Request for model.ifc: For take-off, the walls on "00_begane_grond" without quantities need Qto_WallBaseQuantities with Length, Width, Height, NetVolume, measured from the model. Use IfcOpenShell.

First a look at what the model holds.

```python
import ifcopenshell
import ifcopenshell.util.element
import ifcopenshell.util.unit

model = ifcopenshell.open("model.ifc")
print(model.schema)
for unit_type in ("LENGTHUNIT", "AREAUNIT", "VOLUMEUNIT"):
    print(unit_type, ifcopenshell.util.unit.calculate_unit_scale(model, unit_type))
storey = next(s for s in model.by_type("IfcBuildingStorey") if s.Name == "00_begane_grond")
walls = [e for e in ifcopenshell.util.element.get_decomposition(storey) if e.is_a("IfcWall")]
for e in sorted(walls, key=lambda e: e.id()):
    print(e.id(), e.is_a(), e.Name, list(ifcopenshell.util.element.get_psets(e, qtos_only=True)), sep=" | ")
```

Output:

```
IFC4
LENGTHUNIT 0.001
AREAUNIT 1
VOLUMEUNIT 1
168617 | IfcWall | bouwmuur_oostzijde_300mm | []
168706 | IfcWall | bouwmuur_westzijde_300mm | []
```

```python
import ifcopenshell
import ifcopenshell.api.pset
import ifcopenshell.geom
import ifcopenshell.util.element
import ifcopenshell.util.shape
import ifcopenshell.util.unit

model = ifcopenshell.open("model.ifc")
unit_scale = ifcopenshell.util.unit.calculate_unit_scale(model)
volume_scale = ifcopenshell.util.unit.calculate_unit_scale(model, "VOLUMEUNIT")
settings = ifcopenshell.geom.settings()

storey = next(s for s in model.by_type("IfcBuildingStorey") if s.Name == "00_begane_grond")
walls = [e for e in ifcopenshell.util.element.get_decomposition(storey) if e.is_a("IfcWall")]

for e in sorted(walls, key=lambda e: e.id()):
    if ifcopenshell.util.element.get_psets(e, qtos_only=True, should_inherit=False):
        continue
    # Geometry comes back in metres, in the element's own axes.
    shape = ifcopenshell.geom.create_shape(settings, e)
    values = {
        "Length": ifcopenshell.util.shape.get_x(shape.geometry) / unit_scale,
        "Width": ifcopenshell.util.shape.get_y(shape.geometry) / unit_scale,
        "Height": ifcopenshell.util.shape.get_z(shape.geometry) / unit_scale,
        "NetVolume": ifcopenshell.util.shape.get_volume(shape.geometry) / volume_scale,
    }
    qto = ifcopenshell.api.pset.add_qto(model, product=e, name="Qto_WallBaseQuantities")
    ifcopenshell.api.pset.edit_qto(model, qto=qto, properties=values)
    print(e.id(), {k: round(v, 3) for k, v in values.items()})

model.write("model_v2.ifc")
```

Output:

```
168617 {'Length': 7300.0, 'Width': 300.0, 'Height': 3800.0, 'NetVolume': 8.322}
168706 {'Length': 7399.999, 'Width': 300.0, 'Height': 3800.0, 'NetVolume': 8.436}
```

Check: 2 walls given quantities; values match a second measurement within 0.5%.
